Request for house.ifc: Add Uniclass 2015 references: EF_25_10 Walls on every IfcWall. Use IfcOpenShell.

First a look at what the model holds.

```python
import ifcopenshell

model = ifcopenshell.open("house.ifc")
print(model.schema)
print("classifications:", [c.Name for c in model.by_type("IfcClassification")])
for ifc_class in ("IfcDoor", "IfcRoof", "IfcStair", "IfcWall", "IfcWindow"):
    print(ifc_class, len(model.by_type(ifc_class)))
```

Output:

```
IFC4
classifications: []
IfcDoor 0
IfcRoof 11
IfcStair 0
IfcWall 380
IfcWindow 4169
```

```python
import ifcopenshell
import ifcopenshell.api.classification

model = ifcopenshell.open("house.ifc")

system = ifcopenshell.api.classification.add_classification(model, classification="Uniclass 2015")

codes = {
    "IfcWall": ("EF_25_10", "Walls"),
}
for ifc_class, (code, name) in codes.items():
    products = model.by_type(ifc_class)
    ifcopenshell.api.classification.add_reference(
        model, products=products, classification=system, identification=code, name=name
    )
    print(code, len(products))

model.write("house-out.ifc")
```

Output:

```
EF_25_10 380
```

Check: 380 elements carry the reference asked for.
